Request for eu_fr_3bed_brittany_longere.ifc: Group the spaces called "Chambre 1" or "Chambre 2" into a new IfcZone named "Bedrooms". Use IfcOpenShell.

First a look at what the model holds.

```python
import ifcopenshell

model = ifcopenshell.open("eu_fr_3bed_brittany_longere.ifc")
print(model.schema)
seen = {}
for space in model.by_type("IfcSpace"):
    seen[space.LongName] = seen.get(space.LongName, 0) + 1
for name, count in sorted(seen.items(), key=str):
    print(count, "x", name)
print("zones:", [z.Name for z in model.by_type("IfcZone")][:20])
```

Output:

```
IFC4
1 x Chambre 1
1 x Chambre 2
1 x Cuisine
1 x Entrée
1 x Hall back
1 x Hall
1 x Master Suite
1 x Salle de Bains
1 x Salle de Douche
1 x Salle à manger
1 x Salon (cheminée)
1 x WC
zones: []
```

```python
import ifcopenshell
import ifcopenshell.api.group
import ifcopenshell.api.root

model = ifcopenshell.open("eu_fr_3bed_brittany_longere.ifc")

names = {"Chambre 1", "Chambre 2"}
spaces = [s for s in model.by_type("IfcSpace") if s.LongName in names]

zone = ifcopenshell.api.root.create_entity(model, ifc_class="IfcZone", name="Bedrooms")
ifcopenshell.api.group.assign_group(model, products=spaces, group=zone)
print(len(spaces), "spaces in", zone.Name)

model.write("eu_fr_3bed_brittany_longere_updated.ifc")
```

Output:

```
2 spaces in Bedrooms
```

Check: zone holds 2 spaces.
